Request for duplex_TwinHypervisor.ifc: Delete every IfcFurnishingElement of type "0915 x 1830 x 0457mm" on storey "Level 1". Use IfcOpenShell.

First a look at what the model holds.

```python
import ifcopenshell
import ifcopenshell.util.element

model = ifcopenshell.open("duplex_TwinHypervisor.ifc")
print(model.schema)
storey = next(s for s in model.by_type("IfcBuildingStorey") if s.Name == "Level 1")
furniture = [e for e in ifcopenshell.util.element.get_decomposition(storey) if e.is_a("IfcFurnishingElement")]
seen = {}
for e in furniture:
    element_type = ifcopenshell.util.element.get_type(e)
    name = element_type.Name if element_type not in (None, e) else None
    seen[name] = seen.get(name, 0) + 1
for name, count in sorted(seen.items(), key=str):
    print(count, "x", name)
```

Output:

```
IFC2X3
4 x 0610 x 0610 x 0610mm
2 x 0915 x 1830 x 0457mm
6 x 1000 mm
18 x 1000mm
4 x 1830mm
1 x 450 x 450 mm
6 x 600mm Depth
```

```python
import ifcopenshell
import ifcopenshell.api.root
import ifcopenshell.util.element

model = ifcopenshell.open("duplex_TwinHypervisor.ifc")

storey = next(s for s in model.by_type("IfcBuildingStorey") if s.Name == "Level 1")
furniture = [e for e in ifcopenshell.util.element.get_decomposition(storey) if e.is_a("IfcFurnishingElement")]
targets = [e for e in furniture if (t := ifcopenshell.util.element.get_type(e)) not in (None, e) and t.Name == "0915 x 1830 x 0457mm"]

for e in targets:
    ifcopenshell.api.root.remove_product(model, product=e)
print(len(targets), "removed")

model.write("duplex_TwinHypervisor-out.ifc")
```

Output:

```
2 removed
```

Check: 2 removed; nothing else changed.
